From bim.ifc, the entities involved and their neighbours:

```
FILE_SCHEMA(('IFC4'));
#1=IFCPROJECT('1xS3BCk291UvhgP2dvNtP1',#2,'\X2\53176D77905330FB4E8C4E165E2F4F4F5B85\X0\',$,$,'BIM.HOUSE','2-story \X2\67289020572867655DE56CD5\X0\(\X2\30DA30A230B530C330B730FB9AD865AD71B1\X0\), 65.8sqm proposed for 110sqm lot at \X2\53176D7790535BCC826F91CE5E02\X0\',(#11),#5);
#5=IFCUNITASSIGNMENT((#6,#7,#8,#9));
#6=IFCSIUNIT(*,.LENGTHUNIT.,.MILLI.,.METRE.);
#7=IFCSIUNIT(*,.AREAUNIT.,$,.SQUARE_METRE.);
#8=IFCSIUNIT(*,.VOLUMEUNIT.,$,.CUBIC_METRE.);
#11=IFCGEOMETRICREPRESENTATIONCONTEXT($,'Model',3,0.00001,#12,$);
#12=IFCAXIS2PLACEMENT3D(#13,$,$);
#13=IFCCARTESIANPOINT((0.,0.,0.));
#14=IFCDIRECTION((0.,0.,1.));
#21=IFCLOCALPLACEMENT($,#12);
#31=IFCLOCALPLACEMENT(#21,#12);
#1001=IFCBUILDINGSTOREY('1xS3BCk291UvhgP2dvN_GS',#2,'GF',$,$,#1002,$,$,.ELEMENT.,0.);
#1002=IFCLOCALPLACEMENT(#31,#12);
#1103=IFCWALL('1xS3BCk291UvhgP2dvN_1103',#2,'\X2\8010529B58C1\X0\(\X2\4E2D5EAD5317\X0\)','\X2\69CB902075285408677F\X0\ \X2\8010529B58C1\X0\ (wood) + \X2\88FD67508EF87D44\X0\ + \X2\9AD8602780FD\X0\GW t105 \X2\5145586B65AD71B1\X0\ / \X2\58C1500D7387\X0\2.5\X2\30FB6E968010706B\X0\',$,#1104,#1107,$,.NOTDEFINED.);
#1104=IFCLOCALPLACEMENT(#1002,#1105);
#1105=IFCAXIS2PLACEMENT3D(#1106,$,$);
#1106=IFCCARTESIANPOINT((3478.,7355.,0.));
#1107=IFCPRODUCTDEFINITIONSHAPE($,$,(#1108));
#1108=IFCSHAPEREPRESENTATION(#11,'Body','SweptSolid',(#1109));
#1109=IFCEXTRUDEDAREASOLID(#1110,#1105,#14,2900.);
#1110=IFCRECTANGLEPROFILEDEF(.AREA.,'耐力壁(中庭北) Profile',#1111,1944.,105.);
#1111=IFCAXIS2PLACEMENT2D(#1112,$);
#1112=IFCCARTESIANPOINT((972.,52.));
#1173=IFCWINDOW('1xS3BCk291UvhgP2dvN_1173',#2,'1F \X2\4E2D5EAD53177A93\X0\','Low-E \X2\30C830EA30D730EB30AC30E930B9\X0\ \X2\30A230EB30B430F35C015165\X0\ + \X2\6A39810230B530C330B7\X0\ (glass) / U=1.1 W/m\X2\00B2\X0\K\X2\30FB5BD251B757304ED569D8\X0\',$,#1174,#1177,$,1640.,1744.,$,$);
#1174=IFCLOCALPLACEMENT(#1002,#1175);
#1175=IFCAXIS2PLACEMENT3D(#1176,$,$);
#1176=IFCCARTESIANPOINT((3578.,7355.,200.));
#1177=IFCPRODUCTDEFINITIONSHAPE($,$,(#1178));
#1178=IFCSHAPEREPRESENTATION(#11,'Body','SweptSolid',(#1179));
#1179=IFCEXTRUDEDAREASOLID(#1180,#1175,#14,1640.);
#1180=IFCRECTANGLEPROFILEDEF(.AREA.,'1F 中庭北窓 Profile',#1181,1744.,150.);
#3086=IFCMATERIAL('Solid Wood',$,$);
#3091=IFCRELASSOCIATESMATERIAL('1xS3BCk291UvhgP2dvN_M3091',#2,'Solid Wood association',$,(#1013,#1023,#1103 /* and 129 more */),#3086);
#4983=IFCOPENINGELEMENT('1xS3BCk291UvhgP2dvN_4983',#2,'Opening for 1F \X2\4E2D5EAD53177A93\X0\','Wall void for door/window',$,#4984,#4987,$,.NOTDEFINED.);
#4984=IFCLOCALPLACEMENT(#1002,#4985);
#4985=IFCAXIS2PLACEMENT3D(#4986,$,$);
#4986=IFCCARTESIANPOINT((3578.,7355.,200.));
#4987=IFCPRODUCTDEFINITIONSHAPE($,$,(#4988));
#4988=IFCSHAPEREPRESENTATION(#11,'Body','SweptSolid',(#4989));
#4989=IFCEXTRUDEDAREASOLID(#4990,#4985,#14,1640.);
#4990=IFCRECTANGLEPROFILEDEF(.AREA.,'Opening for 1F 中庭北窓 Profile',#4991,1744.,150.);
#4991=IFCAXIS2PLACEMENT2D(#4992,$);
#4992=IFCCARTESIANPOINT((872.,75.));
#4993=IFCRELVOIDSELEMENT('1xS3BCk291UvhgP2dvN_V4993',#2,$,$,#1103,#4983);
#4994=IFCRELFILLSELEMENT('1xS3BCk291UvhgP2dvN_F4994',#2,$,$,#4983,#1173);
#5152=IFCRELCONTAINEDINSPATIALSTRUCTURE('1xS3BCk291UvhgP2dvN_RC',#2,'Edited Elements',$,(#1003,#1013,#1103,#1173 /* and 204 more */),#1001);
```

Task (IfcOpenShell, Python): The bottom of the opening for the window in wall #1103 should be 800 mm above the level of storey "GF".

```python
import numpy as np
import ifcopenshell
import ifcopenshell.api.geometry
import ifcopenshell.geom
import ifcopenshell.util.element
import ifcopenshell.util.placement
import ifcopenshell.util.shape
import ifcopenshell.util.unit

model = ifcopenshell.open("bim.ifc")
unit_scale = ifcopenshell.util.unit.calculate_unit_scale(model)

window = model.by_guid("1xS3BCk291UvhgP2dvN_1173")
opening = window.FillsVoids[0].RelatingOpeningElement
storey = ifcopenshell.util.element.get_container(window, ifc_class="IfcBuildingStorey")
level = ifcopenshell.util.placement.get_local_placement(storey.ObjectPlacement)[2, 3]

# The opening's origin need not be at the sill, so measure its lowest point.
shape = ifcopenshell.geom.create_shape(ifcopenshell.geom.settings(), opening)
bottom = ifcopenshell.util.shape.get_shape_bottom_elevation(shape, shape.geometry) / unit_scale
dz = level + 0.8 / unit_scale - bottom

shift = np.array([0.0, 0.0, dz])
# The window is not placed relative to its opening, so move both.
for product in (opening, window):
    matrix = ifcopenshell.util.placement.get_local_placement(product.ObjectPlacement)
    matrix[:3, 3] += shift
    ifcopenshell.api.geometry.edit_object_placement(model, product=product, matrix=matrix, is_si=False)

print(f"moved by {dz * unit_scale:+.3f} m")

model.write("bim_v2.ifc")
```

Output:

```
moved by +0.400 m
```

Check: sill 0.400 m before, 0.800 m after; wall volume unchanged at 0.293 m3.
